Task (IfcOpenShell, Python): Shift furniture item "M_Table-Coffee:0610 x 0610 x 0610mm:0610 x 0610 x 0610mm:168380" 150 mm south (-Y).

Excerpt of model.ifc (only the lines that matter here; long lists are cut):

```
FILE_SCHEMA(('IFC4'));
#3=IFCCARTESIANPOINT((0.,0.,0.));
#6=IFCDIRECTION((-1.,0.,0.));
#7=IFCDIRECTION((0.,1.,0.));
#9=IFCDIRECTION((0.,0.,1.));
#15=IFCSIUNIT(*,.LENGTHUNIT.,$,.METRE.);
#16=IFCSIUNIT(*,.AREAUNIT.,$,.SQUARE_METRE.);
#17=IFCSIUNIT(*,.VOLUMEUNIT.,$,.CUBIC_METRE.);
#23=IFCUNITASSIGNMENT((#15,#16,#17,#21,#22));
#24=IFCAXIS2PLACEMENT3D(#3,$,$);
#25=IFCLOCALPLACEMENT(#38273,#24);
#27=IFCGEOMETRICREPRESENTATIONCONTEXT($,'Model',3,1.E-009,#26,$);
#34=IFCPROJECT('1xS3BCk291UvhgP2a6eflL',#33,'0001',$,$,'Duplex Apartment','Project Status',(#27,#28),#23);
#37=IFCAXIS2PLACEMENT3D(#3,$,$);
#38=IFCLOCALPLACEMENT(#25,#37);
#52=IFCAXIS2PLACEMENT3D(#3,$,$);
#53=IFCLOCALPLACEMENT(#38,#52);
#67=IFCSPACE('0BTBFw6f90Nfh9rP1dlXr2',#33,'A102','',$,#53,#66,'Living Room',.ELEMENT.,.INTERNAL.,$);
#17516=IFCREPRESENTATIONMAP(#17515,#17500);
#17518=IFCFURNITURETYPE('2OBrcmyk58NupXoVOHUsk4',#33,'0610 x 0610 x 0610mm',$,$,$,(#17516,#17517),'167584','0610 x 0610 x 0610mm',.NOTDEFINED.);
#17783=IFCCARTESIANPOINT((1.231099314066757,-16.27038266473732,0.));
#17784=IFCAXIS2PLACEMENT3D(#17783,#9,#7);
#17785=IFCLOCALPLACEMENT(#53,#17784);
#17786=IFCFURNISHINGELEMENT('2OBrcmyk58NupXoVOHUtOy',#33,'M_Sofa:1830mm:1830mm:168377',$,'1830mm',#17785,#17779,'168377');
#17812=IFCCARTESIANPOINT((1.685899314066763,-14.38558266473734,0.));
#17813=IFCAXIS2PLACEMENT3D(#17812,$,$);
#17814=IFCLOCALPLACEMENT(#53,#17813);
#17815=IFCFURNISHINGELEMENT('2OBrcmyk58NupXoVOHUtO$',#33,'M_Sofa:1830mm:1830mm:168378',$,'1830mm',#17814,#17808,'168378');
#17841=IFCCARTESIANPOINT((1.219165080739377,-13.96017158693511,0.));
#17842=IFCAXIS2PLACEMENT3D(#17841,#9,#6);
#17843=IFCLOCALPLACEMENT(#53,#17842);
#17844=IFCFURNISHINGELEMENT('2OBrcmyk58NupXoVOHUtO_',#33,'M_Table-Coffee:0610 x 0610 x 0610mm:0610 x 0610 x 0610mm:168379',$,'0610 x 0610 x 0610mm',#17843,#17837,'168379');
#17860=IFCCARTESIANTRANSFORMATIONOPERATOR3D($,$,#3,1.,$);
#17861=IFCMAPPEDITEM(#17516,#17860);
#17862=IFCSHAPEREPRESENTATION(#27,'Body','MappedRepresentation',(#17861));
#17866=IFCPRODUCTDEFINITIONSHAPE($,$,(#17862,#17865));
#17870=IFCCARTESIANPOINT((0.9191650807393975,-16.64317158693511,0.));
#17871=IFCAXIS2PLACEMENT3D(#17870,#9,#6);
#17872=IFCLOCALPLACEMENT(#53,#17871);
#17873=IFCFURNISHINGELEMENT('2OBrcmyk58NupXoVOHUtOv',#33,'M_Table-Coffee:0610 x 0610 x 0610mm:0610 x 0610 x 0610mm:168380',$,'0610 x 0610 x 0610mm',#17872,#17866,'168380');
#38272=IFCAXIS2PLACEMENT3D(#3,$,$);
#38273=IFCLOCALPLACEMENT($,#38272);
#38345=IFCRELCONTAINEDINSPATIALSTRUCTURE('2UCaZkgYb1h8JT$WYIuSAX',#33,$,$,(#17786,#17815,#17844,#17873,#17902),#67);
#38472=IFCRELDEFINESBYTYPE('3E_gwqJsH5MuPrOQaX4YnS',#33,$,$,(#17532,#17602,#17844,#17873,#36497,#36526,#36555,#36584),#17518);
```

```python
import ifcopenshell
import ifcopenshell.api.geometry
import ifcopenshell.util.placement
import ifcopenshell.util.unit

model = ifcopenshell.open("model.ifc")
unit_scale = ifcopenshell.util.unit.calculate_unit_scale(model)

item = model.by_guid("2OBrcmyk58NupXoVOHUtOv")
matrix = ifcopenshell.util.placement.get_local_placement(item.ObjectPlacement)
matrix[1, 3] -= 0.15 / unit_scale
ifcopenshell.api.geometry.edit_object_placement(model, product=item, matrix=matrix, is_si=False)

print(ifcopenshell.util.placement.get_local_placement(item.ObjectPlacement).round(3) + 0.0)

model.write("model_updated.ifc")
```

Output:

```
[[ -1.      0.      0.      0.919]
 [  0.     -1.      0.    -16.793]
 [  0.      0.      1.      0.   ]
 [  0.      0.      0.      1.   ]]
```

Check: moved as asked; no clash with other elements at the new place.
